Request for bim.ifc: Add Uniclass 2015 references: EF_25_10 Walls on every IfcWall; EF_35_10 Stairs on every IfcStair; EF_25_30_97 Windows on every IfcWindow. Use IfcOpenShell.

First a look at what the model holds.

```python
import ifcopenshell

model = ifcopenshell.open("bim.ifc")
print(model.schema)
print("classifications:", [c.Name for c in model.by_type("IfcClassification")])
for ifc_class in ("IfcDoor", "IfcRoof", "IfcStair", "IfcWall", "IfcWindow"):
    print(ifc_class, len(model.by_type(ifc_class)))
```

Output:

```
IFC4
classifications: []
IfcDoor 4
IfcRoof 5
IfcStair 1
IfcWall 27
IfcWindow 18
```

```python
import ifcopenshell
import ifcopenshell.api.classification

model = ifcopenshell.open("bim.ifc")

system = ifcopenshell.api.classification.add_classification(model, classification="Uniclass 2015")

codes = {
    "IfcWall": ("EF_25_10", "Walls"),
    "IfcStair": ("EF_35_10", "Stairs"),
    "IfcWindow": ("EF_25_30_97", "Windows"),
}
for ifc_class, (code, name) in codes.items():
    products = model.by_type(ifc_class)
    ifcopenshell.api.classification.add_reference(
        model, products=products, classification=system, identification=code, name=name
    )
    print(code, len(products))

model.write("bim_edited.ifc")
```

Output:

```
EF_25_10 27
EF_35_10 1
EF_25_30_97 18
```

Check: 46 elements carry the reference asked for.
